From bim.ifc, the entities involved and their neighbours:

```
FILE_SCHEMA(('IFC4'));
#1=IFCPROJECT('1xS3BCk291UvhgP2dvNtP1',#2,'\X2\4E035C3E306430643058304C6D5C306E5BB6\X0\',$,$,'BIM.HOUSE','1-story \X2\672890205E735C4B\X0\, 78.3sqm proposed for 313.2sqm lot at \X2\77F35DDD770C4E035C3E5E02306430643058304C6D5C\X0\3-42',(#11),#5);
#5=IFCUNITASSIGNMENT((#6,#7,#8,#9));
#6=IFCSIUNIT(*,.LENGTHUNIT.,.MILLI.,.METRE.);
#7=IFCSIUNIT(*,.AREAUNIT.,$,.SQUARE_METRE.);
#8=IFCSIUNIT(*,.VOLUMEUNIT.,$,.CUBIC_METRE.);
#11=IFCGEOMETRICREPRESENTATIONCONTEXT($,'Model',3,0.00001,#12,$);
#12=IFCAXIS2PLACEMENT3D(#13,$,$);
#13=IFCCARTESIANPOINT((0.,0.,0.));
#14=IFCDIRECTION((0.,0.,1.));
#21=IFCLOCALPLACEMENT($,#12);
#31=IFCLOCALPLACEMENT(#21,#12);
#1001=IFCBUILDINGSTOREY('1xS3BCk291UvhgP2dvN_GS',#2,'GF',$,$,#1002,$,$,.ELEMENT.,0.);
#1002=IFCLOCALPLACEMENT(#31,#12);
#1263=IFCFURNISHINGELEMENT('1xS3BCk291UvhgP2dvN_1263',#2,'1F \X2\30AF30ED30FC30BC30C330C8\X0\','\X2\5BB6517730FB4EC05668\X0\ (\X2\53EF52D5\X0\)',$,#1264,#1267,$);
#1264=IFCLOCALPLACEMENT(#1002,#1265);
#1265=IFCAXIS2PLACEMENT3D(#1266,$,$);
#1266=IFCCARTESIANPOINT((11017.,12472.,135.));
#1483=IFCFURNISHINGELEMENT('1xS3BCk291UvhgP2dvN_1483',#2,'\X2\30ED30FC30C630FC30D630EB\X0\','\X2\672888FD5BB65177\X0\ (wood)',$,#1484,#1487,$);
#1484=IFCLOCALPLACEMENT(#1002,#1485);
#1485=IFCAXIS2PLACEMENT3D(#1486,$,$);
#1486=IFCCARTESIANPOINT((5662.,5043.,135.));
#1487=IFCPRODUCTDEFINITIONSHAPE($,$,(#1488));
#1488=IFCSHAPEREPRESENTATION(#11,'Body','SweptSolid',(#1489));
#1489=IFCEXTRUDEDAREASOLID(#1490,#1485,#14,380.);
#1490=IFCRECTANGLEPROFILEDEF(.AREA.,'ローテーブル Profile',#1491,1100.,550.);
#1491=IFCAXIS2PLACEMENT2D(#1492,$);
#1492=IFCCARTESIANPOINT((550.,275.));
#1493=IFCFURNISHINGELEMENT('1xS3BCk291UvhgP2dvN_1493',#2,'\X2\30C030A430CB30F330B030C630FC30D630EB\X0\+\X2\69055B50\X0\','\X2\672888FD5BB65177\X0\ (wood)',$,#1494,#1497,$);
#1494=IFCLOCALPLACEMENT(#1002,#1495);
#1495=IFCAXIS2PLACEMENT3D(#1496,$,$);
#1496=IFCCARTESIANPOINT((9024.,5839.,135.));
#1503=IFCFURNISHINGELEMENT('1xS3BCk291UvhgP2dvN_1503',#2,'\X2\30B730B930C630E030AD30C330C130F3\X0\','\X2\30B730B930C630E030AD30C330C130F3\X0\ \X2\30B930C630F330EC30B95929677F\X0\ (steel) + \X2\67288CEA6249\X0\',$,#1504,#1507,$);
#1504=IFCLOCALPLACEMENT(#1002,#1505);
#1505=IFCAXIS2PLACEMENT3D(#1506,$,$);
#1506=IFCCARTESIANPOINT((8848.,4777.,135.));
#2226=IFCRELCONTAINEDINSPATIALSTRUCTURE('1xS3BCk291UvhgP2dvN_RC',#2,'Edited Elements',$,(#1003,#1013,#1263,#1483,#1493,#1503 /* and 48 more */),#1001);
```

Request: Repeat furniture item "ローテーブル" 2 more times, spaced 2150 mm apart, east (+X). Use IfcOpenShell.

```python
import numpy as np
import ifcopenshell
import ifcopenshell.api.geometry
import ifcopenshell.api.root
import ifcopenshell.util.element
import ifcopenshell.util.placement

model = ifcopenshell.open("bim.ifc")


def reuse_history(source, copy):
    """copy_class also copies each property set's owner history, people and application; keep the originals."""
    for rel in copy.IsDefinedBy:
        if rel.is_a("IfcRelDefinesByProperties") and (history := rel.RelatingPropertyDefinition.OwnerHistory):
            rel.RelatingPropertyDefinition.OwnerHistory = source.OwnerHistory
            ifcopenshell.util.element.remove_deep2(model, history)


source = model.by_guid("1xS3BCk291UvhgP2dvN_1483")
base = ifcopenshell.util.placement.get_local_placement(source.ObjectPlacement)
step = np.array([1.0, 0.0, 0.0]) * 2150.0

for i in range(1, 3):
    copy = ifcopenshell.api.root.copy_class(model, product=source)
    copy.Representation = ifcopenshell.util.element.copy_deep(
        model, source.Representation, exclude=["IfcGeometricRepresentationContext", "IfcRepresentationMap"]
    )
    reuse_history(source, copy)
    matrix = base.copy()
    matrix[:3, 3] += i * step
    print("added at", matrix[:3, 3].round(3) + 0.0)
    ifcopenshell.api.geometry.edit_object_placement(model, product=copy, matrix=matrix, is_si=False)

model.write("bim-out.ifc")
```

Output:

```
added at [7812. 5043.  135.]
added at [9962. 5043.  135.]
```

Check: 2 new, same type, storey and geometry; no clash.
